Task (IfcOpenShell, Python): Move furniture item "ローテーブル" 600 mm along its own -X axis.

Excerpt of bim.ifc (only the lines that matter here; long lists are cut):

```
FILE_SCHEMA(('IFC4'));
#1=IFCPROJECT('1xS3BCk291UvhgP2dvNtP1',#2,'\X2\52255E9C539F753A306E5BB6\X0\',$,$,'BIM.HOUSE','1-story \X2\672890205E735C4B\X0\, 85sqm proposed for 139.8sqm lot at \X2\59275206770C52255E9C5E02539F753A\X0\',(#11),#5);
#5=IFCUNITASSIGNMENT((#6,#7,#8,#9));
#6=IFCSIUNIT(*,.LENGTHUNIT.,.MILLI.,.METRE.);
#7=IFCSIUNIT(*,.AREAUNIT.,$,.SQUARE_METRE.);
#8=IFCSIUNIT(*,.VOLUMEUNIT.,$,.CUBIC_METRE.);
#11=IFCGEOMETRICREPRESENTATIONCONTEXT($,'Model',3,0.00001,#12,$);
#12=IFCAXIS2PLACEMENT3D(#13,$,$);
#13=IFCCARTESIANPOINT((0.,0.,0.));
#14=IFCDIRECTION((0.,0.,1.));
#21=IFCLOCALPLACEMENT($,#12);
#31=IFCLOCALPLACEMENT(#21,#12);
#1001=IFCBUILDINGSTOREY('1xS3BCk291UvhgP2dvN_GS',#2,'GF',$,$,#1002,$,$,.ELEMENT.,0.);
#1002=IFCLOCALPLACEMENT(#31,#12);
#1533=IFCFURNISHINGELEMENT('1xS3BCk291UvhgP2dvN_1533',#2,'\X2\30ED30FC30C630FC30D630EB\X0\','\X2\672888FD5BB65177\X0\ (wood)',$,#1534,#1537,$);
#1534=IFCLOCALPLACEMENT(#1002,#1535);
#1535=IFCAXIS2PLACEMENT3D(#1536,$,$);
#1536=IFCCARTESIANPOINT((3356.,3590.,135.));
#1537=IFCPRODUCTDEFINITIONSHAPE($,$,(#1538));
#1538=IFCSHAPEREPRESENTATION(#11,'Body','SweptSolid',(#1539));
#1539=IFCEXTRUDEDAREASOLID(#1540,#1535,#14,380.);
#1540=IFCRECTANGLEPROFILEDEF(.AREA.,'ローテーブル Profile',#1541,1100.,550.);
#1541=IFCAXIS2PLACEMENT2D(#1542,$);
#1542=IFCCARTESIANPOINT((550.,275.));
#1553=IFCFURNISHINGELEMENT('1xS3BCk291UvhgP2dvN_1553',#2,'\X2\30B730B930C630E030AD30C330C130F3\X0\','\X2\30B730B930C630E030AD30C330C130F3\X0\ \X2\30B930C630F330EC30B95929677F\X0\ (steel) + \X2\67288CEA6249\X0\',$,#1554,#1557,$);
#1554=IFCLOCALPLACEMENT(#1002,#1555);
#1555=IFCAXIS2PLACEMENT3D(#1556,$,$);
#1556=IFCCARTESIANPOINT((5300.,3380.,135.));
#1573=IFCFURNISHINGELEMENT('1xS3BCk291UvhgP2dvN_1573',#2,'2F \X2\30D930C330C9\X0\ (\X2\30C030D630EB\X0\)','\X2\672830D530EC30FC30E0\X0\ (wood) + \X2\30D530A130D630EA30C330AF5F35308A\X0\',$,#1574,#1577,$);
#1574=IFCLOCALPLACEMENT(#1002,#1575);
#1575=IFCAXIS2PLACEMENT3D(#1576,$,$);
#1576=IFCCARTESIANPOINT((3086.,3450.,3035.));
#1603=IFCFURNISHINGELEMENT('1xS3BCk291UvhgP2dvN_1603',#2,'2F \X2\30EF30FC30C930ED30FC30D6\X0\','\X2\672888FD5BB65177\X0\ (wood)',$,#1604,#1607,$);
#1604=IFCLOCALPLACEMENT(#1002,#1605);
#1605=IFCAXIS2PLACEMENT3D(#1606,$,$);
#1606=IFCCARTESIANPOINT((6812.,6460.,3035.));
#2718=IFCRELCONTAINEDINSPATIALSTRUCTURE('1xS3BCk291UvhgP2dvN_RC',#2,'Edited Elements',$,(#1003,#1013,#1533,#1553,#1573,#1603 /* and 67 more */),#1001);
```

```python
import ifcopenshell
import ifcopenshell.api.geometry
import ifcopenshell.util.placement

model = ifcopenshell.open("bim.ifc")

item = model.by_guid("1xS3BCk291UvhgP2dvN_1533")
matrix = ifcopenshell.util.placement.get_local_placement(item.ObjectPlacement)
matrix[:3, 3] -= matrix[:3, 0] * 600.0
ifcopenshell.api.geometry.edit_object_placement(model, product=item, matrix=matrix, is_si=False)

print(ifcopenshell.util.placement.get_local_placement(item.ObjectPlacement).round(3) + 0.0)

model.write("bim_edited.ifc")
```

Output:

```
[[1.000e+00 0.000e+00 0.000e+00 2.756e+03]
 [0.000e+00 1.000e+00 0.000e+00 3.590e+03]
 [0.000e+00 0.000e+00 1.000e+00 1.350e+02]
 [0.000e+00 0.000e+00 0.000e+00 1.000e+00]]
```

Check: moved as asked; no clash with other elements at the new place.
